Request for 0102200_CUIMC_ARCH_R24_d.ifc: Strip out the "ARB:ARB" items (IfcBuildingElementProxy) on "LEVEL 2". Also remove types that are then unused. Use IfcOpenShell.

First a look at what the model holds.

```python
import ifcopenshell
import ifcopenshell.util.element

model = ifcopenshell.open("0102200_CUIMC_ARCH_R24_d.ifc")
print(model.schema)
storey = next(s for s in model.by_type("IfcBuildingStorey") if s.Name == "LEVEL 2")
proxies = [e for e in ifcopenshell.util.element.get_decomposition(storey) if e.is_a("IfcBuildingElementProxy")]
seen = {}
for e in proxies:
    element_type = ifcopenshell.util.element.get_type(e)
    name = element_type.Name if element_type not in (None, e) else None
    seen[name] = seen.get(name, 0) + 1
for name, count in sorted(seen.items(), key=str):
    print(count, "x", name)
```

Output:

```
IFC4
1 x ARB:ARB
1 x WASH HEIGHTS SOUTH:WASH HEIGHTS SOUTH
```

```python
import ifcopenshell
import ifcopenshell.api.root
import ifcopenshell.util.element

model = ifcopenshell.open("0102200_CUIMC_ARCH_R24_d.ifc")

storey = next(s for s in model.by_type("IfcBuildingStorey") if s.Name == "LEVEL 2")
proxies = [e for e in ifcopenshell.util.element.get_decomposition(storey) if e.is_a("IfcBuildingElementProxy")]
targets = [e for e in proxies if (t := ifcopenshell.util.element.get_type(e)) not in (None, e) and t.Name == "ARB:ARB"]
types = {ifcopenshell.util.element.get_type(e) for e in targets} - {None, *targets}

for e in targets:
    ifcopenshell.api.root.remove_product(model, product=e)
print(len(targets), "removed")

unused = [t for t in types if not ifcopenshell.util.element.get_types(t)]
for t in unused:
    ifcopenshell.api.root.remove_product(model, product=t)
print(len(unused), "unused types removed")

model.write("0102200_CUIMC_ARCH_R24_d_v2.ifc")
```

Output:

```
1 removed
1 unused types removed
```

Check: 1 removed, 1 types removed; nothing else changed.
